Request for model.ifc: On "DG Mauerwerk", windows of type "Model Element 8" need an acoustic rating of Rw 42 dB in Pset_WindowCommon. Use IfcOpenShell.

First a look at what the model holds.

```python
import ifcopenshell
import ifcopenshell.util.element

model = ifcopenshell.open("model.ifc")
print(model.schema)
storey = next(s for s in model.by_type("IfcBuildingStorey") if s.Name == "DG Mauerwerk")
windows = [e for e in ifcopenshell.util.element.get_decomposition(storey) if e.is_a("IfcWindow")]
seen = {}
for e in windows:
    element_type = ifcopenshell.util.element.get_type(e)
    key = (element_type.Name if element_type != e and element_type else None, ifcopenshell.util.element.get_pset(e, "Pset_WindowCommon", "AcousticRating"))
    seen[key] = seen.get(key, 0) + 1
for (name, value), count in sorted(seen.items(), key=str):
    print(count, "x", name, "|", value)
```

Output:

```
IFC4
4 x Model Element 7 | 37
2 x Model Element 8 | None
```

```python
import ifcopenshell
import ifcopenshell.api.pset
import ifcopenshell.util.element

model = ifcopenshell.open("model.ifc")

storey = next(s for s in model.by_type("IfcBuildingStorey") if s.Name == "DG Mauerwerk")
windows = [e for e in ifcopenshell.util.element.get_decomposition(storey) if e.is_a("IfcWindow")]

count = 0
for e in windows:
    element_type = ifcopenshell.util.element.get_type(e)
    if element_type in (None, e) or element_type.Name != "Model Element 8":
        continue
    # add_pset returns the element's existing set when there is one.
    pset = ifcopenshell.api.pset.add_pset(model, product=e, name="Pset_WindowCommon")
    ifcopenshell.api.pset.edit_pset(model, pset=pset, properties={"AcousticRating": "Rw 42 dB"})
    count += 1

print(count, "windows updated")

model.write("model-out.ifc")
```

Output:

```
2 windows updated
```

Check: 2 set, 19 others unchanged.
